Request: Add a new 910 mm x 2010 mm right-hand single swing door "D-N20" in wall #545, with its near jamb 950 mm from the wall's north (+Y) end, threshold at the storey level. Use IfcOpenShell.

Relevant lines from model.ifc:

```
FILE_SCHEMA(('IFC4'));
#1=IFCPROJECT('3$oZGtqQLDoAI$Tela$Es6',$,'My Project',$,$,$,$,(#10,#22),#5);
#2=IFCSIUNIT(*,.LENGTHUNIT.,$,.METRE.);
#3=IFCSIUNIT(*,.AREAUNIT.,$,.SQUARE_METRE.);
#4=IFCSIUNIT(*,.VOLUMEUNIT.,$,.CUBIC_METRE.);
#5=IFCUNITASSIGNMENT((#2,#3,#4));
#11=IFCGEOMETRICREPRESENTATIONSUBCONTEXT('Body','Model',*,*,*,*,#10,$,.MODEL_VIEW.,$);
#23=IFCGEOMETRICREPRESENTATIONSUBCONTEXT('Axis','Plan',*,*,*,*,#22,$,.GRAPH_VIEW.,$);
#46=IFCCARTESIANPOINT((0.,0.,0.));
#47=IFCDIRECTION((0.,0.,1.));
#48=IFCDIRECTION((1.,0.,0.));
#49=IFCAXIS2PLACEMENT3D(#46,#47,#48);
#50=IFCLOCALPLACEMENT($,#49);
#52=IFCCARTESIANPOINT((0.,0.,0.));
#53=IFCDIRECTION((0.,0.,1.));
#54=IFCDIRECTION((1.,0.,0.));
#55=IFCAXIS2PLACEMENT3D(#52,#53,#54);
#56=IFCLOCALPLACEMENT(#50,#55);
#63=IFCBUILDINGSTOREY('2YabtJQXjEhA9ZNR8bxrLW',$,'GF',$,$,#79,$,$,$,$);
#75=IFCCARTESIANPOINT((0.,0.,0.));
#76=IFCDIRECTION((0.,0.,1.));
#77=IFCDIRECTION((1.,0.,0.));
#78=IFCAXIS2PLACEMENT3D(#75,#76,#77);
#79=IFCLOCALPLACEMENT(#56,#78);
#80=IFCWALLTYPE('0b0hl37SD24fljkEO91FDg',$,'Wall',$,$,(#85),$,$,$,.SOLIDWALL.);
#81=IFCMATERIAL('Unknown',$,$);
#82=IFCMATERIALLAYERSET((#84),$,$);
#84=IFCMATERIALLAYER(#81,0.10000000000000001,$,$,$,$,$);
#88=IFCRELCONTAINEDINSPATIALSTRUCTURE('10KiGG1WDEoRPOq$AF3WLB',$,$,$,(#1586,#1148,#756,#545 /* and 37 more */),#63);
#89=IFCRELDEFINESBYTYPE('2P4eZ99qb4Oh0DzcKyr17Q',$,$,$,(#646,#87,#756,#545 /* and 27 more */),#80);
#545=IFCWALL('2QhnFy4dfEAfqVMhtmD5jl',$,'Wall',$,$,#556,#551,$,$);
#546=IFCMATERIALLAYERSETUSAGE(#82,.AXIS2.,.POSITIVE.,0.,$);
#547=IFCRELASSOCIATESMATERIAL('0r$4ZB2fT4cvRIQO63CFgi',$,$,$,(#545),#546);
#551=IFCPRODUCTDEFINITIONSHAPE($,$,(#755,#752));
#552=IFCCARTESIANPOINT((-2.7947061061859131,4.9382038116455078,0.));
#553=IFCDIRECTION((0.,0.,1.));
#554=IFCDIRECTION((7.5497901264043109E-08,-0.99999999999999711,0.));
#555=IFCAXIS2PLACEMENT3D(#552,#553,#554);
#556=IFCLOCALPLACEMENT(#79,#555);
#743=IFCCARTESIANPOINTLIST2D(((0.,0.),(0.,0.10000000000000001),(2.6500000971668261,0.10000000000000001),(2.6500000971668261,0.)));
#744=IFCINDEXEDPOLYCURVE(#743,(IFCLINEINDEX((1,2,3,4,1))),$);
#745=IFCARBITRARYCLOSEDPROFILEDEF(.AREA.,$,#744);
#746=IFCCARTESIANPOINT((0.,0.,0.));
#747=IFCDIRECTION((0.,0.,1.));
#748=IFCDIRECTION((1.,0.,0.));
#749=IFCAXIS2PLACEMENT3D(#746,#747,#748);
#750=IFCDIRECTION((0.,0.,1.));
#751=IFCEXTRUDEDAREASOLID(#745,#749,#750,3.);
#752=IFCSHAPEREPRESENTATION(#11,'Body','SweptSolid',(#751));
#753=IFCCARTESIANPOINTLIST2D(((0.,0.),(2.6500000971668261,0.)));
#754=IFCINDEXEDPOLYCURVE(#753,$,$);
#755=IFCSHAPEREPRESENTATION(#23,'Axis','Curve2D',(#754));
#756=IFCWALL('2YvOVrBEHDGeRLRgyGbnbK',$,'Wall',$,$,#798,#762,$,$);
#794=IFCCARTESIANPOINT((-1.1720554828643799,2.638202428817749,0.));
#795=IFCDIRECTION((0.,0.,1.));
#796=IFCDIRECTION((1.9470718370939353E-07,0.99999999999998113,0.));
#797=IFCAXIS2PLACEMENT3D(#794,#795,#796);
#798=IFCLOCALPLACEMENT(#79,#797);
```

```python
import numpy as np
import ifcopenshell
import ifcopenshell.api.feature
import ifcopenshell.api.geometry
import ifcopenshell.api.root
import ifcopenshell.api.spatial
import ifcopenshell.geom
import ifcopenshell.util.element
import ifcopenshell.util.placement
import ifcopenshell.util.representation
import ifcopenshell.util.shape
import ifcopenshell.util.unit

model = ifcopenshell.open("model.ifc")
unit_scale = ifcopenshell.util.unit.calculate_unit_scale(model)
settings = ifcopenshell.geom.settings()


def volume(element):
    """Net volume in cubic metres, openings subtracted."""
    shape = ifcopenshell.geom.create_shape(settings, element)
    return ifcopenshell.util.shape.get_volume(shape.geometry)


wall = model.by_guid("2QhnFy4dfEAfqVMhtmD5jl")
storey = ifcopenshell.util.element.get_container(wall, ifc_class="IfcBuildingStorey")
context = ifcopenshell.util.representation.get_context(model, "Model", "Body", "MODEL_VIEW")
before = volume(wall)

width, height, from_end, sill = 0.91, 2.01, 0.95, 0.0  # metres

# The wall runs along its own X axis, and the end named is its -X end.
wall_shape = ifcopenshell.geom.create_shape(settings, wall)
x, y, z = ifcopenshell.util.shape.get_vertices(wall_shape.geometry).T
start = x.min() + from_end
face, thickness = float(y.min()), float(y.max() - y.min())
wall_matrix = ifcopenshell.util.placement.get_local_placement(wall.ObjectPlacement)
level = ifcopenshell.util.placement.get_local_placement(storey.ObjectPlacement)[2, 3]


def in_wall(x, y):
    """Placement at x, y metres in the wall's axes, at sill height."""
    matrix = wall_matrix.copy()
    matrix[:, 3] = wall_matrix @ np.array([x / unit_scale, y / unit_scale, 0.0, 1.0])
    matrix[2, 3] = level + sill / unit_scale
    return matrix


# Opening: a box that overshoots both wall faces by 50 mm.
opening = ifcopenshell.api.root.create_entity(model, ifc_class="IfcOpeningElement", predefined_type="OPENING")
box = ifcopenshell.api.geometry.add_wall_representation(
    model, context=context, length=width, height=height, thickness=thickness + 0.1
)
ifcopenshell.api.geometry.assign_representation(model, product=opening, representation=box)
ifcopenshell.api.geometry.edit_object_placement(model, product=opening, matrix=in_wall(start, face - 0.05), is_si=False)
ifcopenshell.api.feature.add_feature(model, feature=opening, element=wall)

door = ifcopenshell.api.root.create_entity(model, ifc_class="IfcDoor", name="D-N20", predefined_type="DOOR")
door.OverallWidth, door.OverallHeight = width / unit_scale, height / unit_scale
door.OperationType = "SINGLE_SWING_RIGHT"
body = ifcopenshell.api.geometry.add_door_representation(
    model,
    context=context,
    overall_width=door.OverallWidth,
    overall_height=door.OverallHeight,
    operation_type="SINGLE_SWING_RIGHT",
    lining_properties={"LiningDepth": thickness / unit_scale, "ThresholdDepth": thickness / unit_scale},
)
ifcopenshell.api.geometry.assign_representation(model, product=door, representation=body)
ifcopenshell.api.spatial.assign_container(model, products=[door], relating_structure=storey)
ifcopenshell.api.feature.add_filling(model, opening=opening, element=door)

# The lining spans the wall, so the door starts at the wall face.
ifcopenshell.api.geometry.edit_object_placement(model, product=door, matrix=in_wall(start, face), is_si=False)

after = volume(wall)

print(f"wall volume {before:.3f} -> {after:.3f} m3")

model.write("model_updated.ifc")
```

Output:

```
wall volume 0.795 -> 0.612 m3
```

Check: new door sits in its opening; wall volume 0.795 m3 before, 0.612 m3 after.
